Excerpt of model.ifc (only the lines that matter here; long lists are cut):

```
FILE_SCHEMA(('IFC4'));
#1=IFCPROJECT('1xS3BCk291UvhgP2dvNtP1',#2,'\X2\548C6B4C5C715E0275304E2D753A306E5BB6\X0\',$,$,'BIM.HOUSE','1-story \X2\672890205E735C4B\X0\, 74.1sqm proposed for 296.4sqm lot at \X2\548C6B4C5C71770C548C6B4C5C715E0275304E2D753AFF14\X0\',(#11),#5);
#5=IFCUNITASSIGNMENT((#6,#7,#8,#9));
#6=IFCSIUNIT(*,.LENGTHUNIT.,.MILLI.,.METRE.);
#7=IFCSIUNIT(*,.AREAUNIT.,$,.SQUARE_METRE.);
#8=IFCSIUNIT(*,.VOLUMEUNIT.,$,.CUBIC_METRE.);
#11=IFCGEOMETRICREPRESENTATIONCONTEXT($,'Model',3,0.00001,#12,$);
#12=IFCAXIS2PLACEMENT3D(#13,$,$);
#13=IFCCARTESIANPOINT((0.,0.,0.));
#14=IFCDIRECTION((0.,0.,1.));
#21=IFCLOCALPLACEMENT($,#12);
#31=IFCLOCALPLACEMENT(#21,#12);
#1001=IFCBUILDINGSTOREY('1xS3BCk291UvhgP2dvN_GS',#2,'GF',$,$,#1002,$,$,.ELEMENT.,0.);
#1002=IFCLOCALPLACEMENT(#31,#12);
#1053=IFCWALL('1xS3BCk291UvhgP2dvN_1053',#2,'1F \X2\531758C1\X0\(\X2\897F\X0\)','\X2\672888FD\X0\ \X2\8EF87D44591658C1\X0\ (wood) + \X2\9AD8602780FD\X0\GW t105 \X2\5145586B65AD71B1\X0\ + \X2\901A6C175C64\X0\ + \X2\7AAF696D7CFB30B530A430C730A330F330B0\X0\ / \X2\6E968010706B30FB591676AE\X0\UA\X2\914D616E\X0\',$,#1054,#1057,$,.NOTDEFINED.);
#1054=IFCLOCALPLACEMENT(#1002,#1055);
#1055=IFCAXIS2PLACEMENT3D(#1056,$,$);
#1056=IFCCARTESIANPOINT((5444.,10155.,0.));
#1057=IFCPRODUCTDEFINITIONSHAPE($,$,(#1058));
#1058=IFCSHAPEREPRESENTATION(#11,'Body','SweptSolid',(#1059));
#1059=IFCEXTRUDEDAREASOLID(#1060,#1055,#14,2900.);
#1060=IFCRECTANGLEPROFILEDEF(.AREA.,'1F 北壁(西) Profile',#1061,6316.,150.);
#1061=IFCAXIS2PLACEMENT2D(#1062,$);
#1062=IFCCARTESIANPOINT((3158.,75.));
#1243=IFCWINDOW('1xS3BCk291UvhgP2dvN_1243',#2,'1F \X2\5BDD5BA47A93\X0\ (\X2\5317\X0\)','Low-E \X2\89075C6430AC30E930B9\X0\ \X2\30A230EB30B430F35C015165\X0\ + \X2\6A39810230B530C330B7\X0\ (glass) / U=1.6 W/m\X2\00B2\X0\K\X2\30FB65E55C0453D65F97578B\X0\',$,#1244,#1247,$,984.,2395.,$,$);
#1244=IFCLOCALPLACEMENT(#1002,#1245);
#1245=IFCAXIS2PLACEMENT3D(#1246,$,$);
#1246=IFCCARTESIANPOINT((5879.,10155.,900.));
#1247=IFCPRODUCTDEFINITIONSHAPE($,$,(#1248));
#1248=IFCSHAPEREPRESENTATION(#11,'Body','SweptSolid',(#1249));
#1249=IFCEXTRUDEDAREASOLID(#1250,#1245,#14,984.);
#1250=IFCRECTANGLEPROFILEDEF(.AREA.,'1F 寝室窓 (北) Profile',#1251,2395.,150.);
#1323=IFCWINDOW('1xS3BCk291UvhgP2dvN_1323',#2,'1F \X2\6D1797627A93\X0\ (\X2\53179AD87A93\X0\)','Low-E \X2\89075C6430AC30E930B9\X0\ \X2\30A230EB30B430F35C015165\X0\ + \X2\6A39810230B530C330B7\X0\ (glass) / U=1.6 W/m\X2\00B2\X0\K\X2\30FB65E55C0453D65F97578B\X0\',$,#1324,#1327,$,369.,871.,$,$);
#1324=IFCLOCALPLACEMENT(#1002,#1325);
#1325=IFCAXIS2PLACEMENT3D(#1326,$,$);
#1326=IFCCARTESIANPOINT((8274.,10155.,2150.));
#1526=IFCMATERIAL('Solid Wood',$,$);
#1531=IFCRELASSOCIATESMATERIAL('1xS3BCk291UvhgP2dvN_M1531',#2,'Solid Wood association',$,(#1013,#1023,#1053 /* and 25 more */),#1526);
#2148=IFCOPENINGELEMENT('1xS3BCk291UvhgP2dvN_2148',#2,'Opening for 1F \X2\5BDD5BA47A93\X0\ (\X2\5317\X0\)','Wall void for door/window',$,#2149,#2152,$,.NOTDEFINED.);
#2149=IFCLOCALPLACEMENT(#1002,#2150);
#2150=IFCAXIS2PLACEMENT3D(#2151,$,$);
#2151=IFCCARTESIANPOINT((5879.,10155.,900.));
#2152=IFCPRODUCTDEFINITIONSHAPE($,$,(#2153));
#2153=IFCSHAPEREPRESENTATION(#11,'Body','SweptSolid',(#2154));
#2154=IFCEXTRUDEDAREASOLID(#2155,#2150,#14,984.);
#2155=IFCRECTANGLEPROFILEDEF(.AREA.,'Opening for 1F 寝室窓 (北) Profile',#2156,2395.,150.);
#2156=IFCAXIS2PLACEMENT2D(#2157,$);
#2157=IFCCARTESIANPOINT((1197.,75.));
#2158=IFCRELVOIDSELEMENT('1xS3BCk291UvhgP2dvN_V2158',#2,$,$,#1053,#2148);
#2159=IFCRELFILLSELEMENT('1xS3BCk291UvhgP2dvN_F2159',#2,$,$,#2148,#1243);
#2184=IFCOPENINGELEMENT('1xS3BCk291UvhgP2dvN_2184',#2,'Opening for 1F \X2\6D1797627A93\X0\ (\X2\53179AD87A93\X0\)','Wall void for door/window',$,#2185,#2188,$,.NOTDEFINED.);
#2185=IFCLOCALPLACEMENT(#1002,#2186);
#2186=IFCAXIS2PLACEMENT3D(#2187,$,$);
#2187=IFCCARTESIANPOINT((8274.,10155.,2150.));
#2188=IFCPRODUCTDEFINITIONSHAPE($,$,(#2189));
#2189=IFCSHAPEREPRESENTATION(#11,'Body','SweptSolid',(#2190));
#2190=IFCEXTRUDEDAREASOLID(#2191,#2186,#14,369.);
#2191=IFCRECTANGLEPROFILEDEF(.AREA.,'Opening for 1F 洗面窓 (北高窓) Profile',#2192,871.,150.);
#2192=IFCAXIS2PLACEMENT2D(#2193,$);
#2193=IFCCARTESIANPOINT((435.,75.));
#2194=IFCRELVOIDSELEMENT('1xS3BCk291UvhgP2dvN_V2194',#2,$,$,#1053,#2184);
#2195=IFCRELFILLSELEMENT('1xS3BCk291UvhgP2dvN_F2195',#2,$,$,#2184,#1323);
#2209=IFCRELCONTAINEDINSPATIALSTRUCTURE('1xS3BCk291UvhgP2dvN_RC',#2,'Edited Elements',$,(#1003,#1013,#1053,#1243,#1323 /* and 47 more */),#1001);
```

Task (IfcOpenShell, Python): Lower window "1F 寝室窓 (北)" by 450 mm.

```python
import numpy as np
import ifcopenshell
import ifcopenshell.api.geometry
import ifcopenshell.util.placement
import ifcopenshell.util.unit

model = ifcopenshell.open("model.ifc")
unit_scale = ifcopenshell.util.unit.calculate_unit_scale(model)

window = model.by_id(1243)
opening = window.FillsVoids[0].RelatingOpeningElement
dz = -0.45 / unit_scale

shift = np.array([0.0, 0.0, dz])
# The window is not placed relative to its opening, so move both.
for product in (opening, window):
    matrix = ifcopenshell.util.placement.get_local_placement(product.ObjectPlacement)
    matrix[:3, 3] += shift
    ifcopenshell.api.geometry.edit_object_placement(model, product=product, matrix=matrix, is_si=False)

print(f"moved by {dz * unit_scale:+.3f} m")

model.write("model-out.ifc")
```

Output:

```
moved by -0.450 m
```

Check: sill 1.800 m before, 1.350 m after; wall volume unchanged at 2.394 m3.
